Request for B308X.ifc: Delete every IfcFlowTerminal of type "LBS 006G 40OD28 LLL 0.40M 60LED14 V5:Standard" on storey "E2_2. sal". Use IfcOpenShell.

First a look at what the model holds.

```python
import ifcopenshell
import ifcopenshell.util.element

model = ifcopenshell.open("B308X.ifc")
print(model.schema)
storey = next(s for s in model.by_type("IfcBuildingStorey") if s.Name == "E2_2. sal")
terminals = [e for e in ifcopenshell.util.element.get_decomposition(storey) if e.is_a("IfcFlowTerminal")]
seen = {}
for e in terminals:
    element_type = ifcopenshell.util.element.get_type(e)
    name = element_type.Name if element_type not in (None, e) else None
    seen[name] = seen.get(name, 0) + 1
for name, count in sorted(seen.items(), key=str):
    print(count, "x", name)
```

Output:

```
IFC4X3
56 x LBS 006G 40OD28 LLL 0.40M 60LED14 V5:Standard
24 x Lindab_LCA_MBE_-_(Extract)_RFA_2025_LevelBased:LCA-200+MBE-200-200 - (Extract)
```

```python
import ifcopenshell
import ifcopenshell.api.root
import ifcopenshell.util.element

model = ifcopenshell.open("B308X.ifc")

storey = next(s for s in model.by_type("IfcBuildingStorey") if s.Name == "E2_2. sal")
terminals = [e for e in ifcopenshell.util.element.get_decomposition(storey) if e.is_a("IfcFlowTerminal")]
targets = [e for e in terminals if (t := ifcopenshell.util.element.get_type(e)) not in (None, e) and t.Name == "LBS 006G 40OD28 LLL 0.40M 60LED14 V5:Standard"]

for e in targets:
    ifcopenshell.api.root.remove_product(model, product=e)
print(len(targets), "removed")

model.write("B308X_rev.ifc")
```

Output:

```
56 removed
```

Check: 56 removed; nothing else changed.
